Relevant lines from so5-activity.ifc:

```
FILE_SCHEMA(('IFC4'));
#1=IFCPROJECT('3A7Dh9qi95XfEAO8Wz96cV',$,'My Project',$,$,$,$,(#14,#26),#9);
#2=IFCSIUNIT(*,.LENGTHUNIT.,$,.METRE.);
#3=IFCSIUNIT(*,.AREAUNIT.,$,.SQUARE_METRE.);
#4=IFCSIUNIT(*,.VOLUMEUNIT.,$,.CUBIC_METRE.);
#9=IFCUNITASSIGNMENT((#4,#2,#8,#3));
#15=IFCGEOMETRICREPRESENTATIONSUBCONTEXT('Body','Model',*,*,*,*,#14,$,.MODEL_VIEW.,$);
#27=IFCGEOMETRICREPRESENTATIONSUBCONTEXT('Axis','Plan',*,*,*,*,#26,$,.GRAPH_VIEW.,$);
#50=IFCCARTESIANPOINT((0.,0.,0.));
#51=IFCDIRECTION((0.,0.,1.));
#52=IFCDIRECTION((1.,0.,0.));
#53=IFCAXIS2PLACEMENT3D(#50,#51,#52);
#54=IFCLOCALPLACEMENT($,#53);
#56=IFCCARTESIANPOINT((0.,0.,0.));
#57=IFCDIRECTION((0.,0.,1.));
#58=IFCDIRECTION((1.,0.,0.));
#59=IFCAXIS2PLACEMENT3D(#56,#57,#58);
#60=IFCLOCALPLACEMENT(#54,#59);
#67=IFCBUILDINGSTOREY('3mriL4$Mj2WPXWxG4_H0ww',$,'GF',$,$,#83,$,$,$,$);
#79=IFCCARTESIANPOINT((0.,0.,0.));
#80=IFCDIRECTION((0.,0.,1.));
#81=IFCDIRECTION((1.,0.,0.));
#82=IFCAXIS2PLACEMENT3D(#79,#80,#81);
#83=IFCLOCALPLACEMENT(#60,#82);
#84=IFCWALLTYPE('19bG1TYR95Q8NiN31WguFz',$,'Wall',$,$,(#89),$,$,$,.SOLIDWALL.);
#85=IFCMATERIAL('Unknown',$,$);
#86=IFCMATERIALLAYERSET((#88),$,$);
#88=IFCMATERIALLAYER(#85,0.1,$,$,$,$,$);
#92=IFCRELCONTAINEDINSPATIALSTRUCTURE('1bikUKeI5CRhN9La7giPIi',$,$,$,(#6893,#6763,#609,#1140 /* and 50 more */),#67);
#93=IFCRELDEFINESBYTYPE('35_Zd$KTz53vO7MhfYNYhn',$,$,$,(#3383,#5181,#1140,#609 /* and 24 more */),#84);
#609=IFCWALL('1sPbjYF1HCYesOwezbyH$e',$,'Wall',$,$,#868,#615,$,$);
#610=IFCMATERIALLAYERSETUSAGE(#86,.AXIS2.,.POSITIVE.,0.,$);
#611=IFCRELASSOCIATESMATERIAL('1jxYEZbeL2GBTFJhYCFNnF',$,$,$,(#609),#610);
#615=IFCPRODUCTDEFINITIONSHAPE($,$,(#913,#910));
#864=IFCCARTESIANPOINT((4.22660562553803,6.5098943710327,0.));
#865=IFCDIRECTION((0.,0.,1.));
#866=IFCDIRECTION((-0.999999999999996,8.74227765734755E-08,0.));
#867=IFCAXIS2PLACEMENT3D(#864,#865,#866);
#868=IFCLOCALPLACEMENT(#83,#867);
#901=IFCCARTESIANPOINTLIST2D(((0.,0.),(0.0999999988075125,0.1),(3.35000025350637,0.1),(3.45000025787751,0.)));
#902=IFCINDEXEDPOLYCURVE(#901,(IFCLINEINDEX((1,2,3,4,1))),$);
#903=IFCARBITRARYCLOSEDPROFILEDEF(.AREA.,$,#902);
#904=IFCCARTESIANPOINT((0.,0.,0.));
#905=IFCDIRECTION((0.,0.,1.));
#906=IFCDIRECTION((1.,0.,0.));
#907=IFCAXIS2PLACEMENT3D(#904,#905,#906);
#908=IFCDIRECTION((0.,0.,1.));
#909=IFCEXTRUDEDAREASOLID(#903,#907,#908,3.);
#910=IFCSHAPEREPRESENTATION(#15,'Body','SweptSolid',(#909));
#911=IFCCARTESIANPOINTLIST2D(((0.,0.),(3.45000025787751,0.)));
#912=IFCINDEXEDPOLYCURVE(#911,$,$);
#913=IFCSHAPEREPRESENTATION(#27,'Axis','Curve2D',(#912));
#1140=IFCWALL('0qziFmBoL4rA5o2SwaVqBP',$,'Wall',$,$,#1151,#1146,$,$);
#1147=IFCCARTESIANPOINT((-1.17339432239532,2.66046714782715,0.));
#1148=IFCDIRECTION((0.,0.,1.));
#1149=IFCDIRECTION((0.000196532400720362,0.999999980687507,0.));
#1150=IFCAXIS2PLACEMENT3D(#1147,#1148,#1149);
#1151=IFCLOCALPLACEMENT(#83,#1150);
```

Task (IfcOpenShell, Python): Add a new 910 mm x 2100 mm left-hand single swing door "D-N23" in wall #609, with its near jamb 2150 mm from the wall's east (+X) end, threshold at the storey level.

```python
import numpy as np
import ifcopenshell
import ifcopenshell.api.feature
import ifcopenshell.api.geometry
import ifcopenshell.api.root
import ifcopenshell.api.spatial
import ifcopenshell.geom
import ifcopenshell.util.element
import ifcopenshell.util.placement
import ifcopenshell.util.representation
import ifcopenshell.util.shape
import ifcopenshell.util.unit

model = ifcopenshell.open("so5-activity.ifc")
unit_scale = ifcopenshell.util.unit.calculate_unit_scale(model)
settings = ifcopenshell.geom.settings()


def volume(element):
    """Net volume in cubic metres, openings subtracted."""
    shape = ifcopenshell.geom.create_shape(settings, element)
    return ifcopenshell.util.shape.get_volume(shape.geometry)


wall = model.by_guid("1sPbjYF1HCYesOwezbyH$e")
storey = ifcopenshell.util.element.get_container(wall, ifc_class="IfcBuildingStorey")
context = ifcopenshell.util.representation.get_context(model, "Model", "Body", "MODEL_VIEW")
before = volume(wall)

width, height, from_end, sill = 0.91, 2.1, 2.15, 0.0  # metres

# The wall runs along its own X axis, and the end named is its -X end.
wall_shape = ifcopenshell.geom.create_shape(settings, wall)
x, y, z = ifcopenshell.util.shape.get_vertices(wall_shape.geometry).T
start = x.min() + from_end
face, thickness = float(y.min()), float(y.max() - y.min())
wall_matrix = ifcopenshell.util.placement.get_local_placement(wall.ObjectPlacement)
level = ifcopenshell.util.placement.get_local_placement(storey.ObjectPlacement)[2, 3]


def in_wall(x, y):
    """Placement at x, y metres in the wall's axes, at sill height."""
    matrix = wall_matrix.copy()
    matrix[:, 3] = wall_matrix @ np.array([x / unit_scale, y / unit_scale, 0.0, 1.0])
    matrix[2, 3] = level + sill / unit_scale
    return matrix


# Opening: a box that overshoots both wall faces by 50 mm.
opening = ifcopenshell.api.root.create_entity(model, ifc_class="IfcOpeningElement", predefined_type="OPENING")
box = ifcopenshell.api.geometry.add_wall_representation(
    model, context=context, length=width, height=height, thickness=thickness + 0.1
)
ifcopenshell.api.geometry.assign_representation(model, product=opening, representation=box)
ifcopenshell.api.geometry.edit_object_placement(model, product=opening, matrix=in_wall(start, face - 0.05), is_si=False)
ifcopenshell.api.feature.add_feature(model, feature=opening, element=wall)

door = ifcopenshell.api.root.create_entity(model, ifc_class="IfcDoor", name="D-N23", predefined_type="DOOR")
door.OverallWidth, door.OverallHeight = width / unit_scale, height / unit_scale
door.OperationType = "SINGLE_SWING_LEFT"
body = ifcopenshell.api.geometry.add_door_representation(
    model,
    context=context,
    overall_width=door.OverallWidth,
    overall_height=door.OverallHeight,
    operation_type="SINGLE_SWING_LEFT",
    lining_properties={"LiningDepth": thickness / unit_scale, "ThresholdDepth": thickness / unit_scale},
)
ifcopenshell.api.geometry.assign_representation(model, product=door, representation=body)
ifcopenshell.api.spatial.assign_container(model, products=[door], relating_structure=storey)
ifcopenshell.api.feature.add_filling(model, opening=opening, element=door)

# The lining spans the wall, so the door starts at the wall face.
ifcopenshell.api.geometry.edit_object_placement(model, product=door, matrix=in_wall(start, face), is_si=False)

after = volume(wall)

print(f"wall volume {before:.3f} -> {after:.3f} m3")

model.write("so5-activity-out.ifc")
```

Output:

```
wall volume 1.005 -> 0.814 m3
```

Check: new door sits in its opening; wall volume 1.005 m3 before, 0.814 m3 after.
